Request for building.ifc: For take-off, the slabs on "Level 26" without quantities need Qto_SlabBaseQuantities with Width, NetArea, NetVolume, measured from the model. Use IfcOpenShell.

First a look at what the model holds.

```python
import ifcopenshell
import ifcopenshell.util.element
import ifcopenshell.util.unit

model = ifcopenshell.open("building.ifc")
print(model.schema)
for unit_type in ("LENGTHUNIT", "AREAUNIT", "VOLUMEUNIT"):
    print(unit_type, ifcopenshell.util.unit.calculate_unit_scale(model, unit_type))
storey = next(s for s in model.by_type("IfcBuildingStorey") if s.Name == "Level 26")
slabs = [e for e in ifcopenshell.util.element.get_decomposition(storey) if e.is_a("IfcSlab")]
for e in sorted(slabs, key=lambda e: e.id()):
    print(e.id(), e.is_a(), e.Name, list(ifcopenshell.util.element.get_psets(e, qtos_only=True)), sep=" | ")
```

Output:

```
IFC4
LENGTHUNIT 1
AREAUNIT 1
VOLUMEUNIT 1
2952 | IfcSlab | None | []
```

```python
import ifcopenshell
import ifcopenshell.api.pset
import ifcopenshell.geom
import ifcopenshell.util.element
import ifcopenshell.util.shape
import ifcopenshell.util.unit

model = ifcopenshell.open("building.ifc")
unit_scale = ifcopenshell.util.unit.calculate_unit_scale(model)
area_scale = ifcopenshell.util.unit.calculate_unit_scale(model, "AREAUNIT")
volume_scale = ifcopenshell.util.unit.calculate_unit_scale(model, "VOLUMEUNIT")
settings = ifcopenshell.geom.settings()

storey = next(s for s in model.by_type("IfcBuildingStorey") if s.Name == "Level 26")
slabs = [e for e in ifcopenshell.util.element.get_decomposition(storey) if e.is_a("IfcSlab")]

for e in sorted(slabs, key=lambda e: e.id()):
    if ifcopenshell.util.element.get_psets(e, qtos_only=True, should_inherit=False):
        continue
    # Geometry comes back in metres, in the element's own axes.
    shape = ifcopenshell.geom.create_shape(settings, e)
    values = {
        "Width": ifcopenshell.util.shape.get_z(shape.geometry) / unit_scale,
        "NetArea": ifcopenshell.util.shape.get_footprint_area(shape.geometry) / area_scale,
        "NetVolume": ifcopenshell.util.shape.get_volume(shape.geometry) / volume_scale,
    }
    qto = ifcopenshell.api.pset.add_qto(model, product=e, name="Qto_SlabBaseQuantities")
    ifcopenshell.api.pset.edit_qto(model, qto=qto, properties=values)
    print(e.id(), {k: round(v, 3) for k, v in values.items()})

model.write("building_edited.ifc")
```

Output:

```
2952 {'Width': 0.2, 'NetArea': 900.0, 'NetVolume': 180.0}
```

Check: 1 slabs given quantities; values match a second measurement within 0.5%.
